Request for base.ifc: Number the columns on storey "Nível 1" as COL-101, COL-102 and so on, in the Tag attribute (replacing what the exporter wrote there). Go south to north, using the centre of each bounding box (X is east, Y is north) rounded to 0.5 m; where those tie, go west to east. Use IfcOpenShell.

First a look at what the model holds.

```python
import ifcopenshell
import ifcopenshell.util.element
import ifcopenshell.util.placement

model = ifcopenshell.open("base.ifc")
print(model.schema)
storey = next(s for s in model.by_type("IfcBuildingStorey") if s.Name == "Nível 1")
columns = [e for e in ifcopenshell.util.element.get_decomposition(storey) if e.is_a("IfcColumn")]
for e in sorted(columns, key=lambda e: e.id()):
    origin = ifcopenshell.util.placement.get_local_placement(e.ObjectPlacement)[:3, 3]
    print(e.id(), e.Tag, e.Name, origin.round(2) + 0.0, sep=" | ")
```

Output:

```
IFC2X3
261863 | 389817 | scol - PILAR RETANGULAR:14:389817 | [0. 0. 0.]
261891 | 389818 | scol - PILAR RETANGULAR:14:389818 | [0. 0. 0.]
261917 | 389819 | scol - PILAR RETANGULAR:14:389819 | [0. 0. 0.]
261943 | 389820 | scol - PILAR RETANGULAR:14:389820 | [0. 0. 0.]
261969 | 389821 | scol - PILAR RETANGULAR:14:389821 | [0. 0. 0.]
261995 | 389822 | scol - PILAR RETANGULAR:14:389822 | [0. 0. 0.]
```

```python
import ifcopenshell
import ifcopenshell.geom
import ifcopenshell.util.element
import ifcopenshell.util.shape

model = ifcopenshell.open("base.ifc")
settings = ifcopenshell.geom.settings()
settings.set("use-world-coords", True)


def centre(element):
    shape = ifcopenshell.geom.create_shape(settings, element)
    return ifcopenshell.util.shape.get_bbox_centroid(shape.geometry)


storey = next(s for s in model.by_type("IfcBuildingStorey") if s.Name == "Nível 1")
columns = [e for e in ifcopenshell.util.element.get_decomposition(storey) if e.is_a("IfcColumn")]

# Insertion points can sit at a corner or the storey origin, so sort by the geometry (in metres).
centres = {e: centre(e) for e in columns}
columns.sort(key=lambda e: (round(centres[e][1] / 0.5), centres[e][0]))

for i, e in enumerate(columns, start=1):
    number = f"COL-1{i:02d}"
    e.Tag = number
    print(e.id(), number)

model.write("base_updated.ifc")
```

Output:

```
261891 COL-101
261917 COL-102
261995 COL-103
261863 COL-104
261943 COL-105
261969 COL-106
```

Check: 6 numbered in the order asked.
